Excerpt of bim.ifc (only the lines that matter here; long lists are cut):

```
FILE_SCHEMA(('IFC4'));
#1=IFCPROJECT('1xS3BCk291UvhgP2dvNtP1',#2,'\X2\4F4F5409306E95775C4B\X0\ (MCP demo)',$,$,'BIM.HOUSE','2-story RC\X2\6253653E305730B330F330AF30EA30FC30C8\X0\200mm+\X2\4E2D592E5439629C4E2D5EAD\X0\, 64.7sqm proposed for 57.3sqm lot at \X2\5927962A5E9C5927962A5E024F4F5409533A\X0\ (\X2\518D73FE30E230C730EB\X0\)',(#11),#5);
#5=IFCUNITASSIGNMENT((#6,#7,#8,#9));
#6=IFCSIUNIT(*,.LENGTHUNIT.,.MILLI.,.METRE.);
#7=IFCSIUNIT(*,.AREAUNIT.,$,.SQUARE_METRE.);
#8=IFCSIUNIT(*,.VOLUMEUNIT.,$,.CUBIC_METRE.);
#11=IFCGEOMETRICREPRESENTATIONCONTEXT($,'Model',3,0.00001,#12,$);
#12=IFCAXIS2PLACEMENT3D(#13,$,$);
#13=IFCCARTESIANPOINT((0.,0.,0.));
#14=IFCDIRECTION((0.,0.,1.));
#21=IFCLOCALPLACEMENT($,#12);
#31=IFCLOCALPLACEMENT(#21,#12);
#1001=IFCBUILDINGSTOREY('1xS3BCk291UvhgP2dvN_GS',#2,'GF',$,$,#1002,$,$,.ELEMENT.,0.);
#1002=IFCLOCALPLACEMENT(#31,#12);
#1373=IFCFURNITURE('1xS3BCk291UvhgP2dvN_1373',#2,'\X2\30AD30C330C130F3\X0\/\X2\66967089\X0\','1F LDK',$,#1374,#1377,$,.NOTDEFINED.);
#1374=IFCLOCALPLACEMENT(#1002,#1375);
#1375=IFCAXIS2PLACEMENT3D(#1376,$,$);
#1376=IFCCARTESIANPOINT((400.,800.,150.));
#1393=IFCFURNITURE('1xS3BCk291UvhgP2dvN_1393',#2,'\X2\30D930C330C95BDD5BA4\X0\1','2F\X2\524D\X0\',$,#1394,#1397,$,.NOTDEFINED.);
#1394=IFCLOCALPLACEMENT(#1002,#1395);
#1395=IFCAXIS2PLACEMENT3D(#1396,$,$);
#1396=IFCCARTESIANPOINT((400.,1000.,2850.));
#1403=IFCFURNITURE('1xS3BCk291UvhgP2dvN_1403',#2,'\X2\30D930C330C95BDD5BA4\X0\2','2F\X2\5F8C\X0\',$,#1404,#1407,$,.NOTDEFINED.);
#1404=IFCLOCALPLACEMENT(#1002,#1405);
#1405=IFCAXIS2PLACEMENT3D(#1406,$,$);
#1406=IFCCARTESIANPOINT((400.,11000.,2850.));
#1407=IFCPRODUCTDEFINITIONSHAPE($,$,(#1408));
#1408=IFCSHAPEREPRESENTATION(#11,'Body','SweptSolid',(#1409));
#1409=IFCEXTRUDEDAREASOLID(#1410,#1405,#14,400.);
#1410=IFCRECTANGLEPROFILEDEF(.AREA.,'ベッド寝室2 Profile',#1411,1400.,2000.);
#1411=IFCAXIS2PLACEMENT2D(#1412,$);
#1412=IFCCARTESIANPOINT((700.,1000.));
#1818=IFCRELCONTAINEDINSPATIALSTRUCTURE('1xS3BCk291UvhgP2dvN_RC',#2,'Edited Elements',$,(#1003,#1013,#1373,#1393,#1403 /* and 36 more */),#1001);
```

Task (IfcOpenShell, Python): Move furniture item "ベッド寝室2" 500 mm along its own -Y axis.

```python
import ifcopenshell
import ifcopenshell.api.geometry
import ifcopenshell.util.placement
import ifcopenshell.util.unit

model = ifcopenshell.open("bim.ifc")
unit_scale = ifcopenshell.util.unit.calculate_unit_scale(model)

item = model.by_guid("1xS3BCk291UvhgP2dvN_1403")
matrix = ifcopenshell.util.placement.get_local_placement(item.ObjectPlacement)
matrix[:3, 3] -= matrix[:3, 1] * 0.5 / unit_scale
ifcopenshell.api.geometry.edit_object_placement(model, product=item, matrix=matrix, is_si=False)

print(ifcopenshell.util.placement.get_local_placement(item.ObjectPlacement).round(3) + 0.0)

model.write("bim_updated.ifc")
```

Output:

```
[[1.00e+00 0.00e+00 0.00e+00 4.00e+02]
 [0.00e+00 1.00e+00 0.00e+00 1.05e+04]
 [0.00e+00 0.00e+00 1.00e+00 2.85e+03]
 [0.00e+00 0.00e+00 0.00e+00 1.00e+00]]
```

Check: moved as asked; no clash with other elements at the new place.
